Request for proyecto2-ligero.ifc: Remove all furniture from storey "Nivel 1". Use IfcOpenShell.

First a look at what the model holds.

```python
import ifcopenshell
import ifcopenshell.util.element

model = ifcopenshell.open("proyecto2-ligero.ifc")
print(model.schema)
storey = next(s for s in model.by_type("IfcBuildingStorey") if s.Name == "Nivel 1")
furniture = [e for e in ifcopenshell.util.element.get_decomposition(storey) if e.is_a("IfcFurnishingElement")]
seen = {}
for e in furniture:
    element_type = ifcopenshell.util.element.get_type(e)
    name = element_type.Name if element_type not in (None, e) else None
    seen[name] = seen.get(name, 0) + 1
for name, count in sorted(seen.items(), key=str):
    print(count, "x", name)
```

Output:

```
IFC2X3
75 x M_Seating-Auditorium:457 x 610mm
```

```python
import ifcopenshell
import ifcopenshell.api.root
import ifcopenshell.util.element

model = ifcopenshell.open("proyecto2-ligero.ifc")

storey = next(s for s in model.by_type("IfcBuildingStorey") if s.Name == "Nivel 1")
furniture = [e for e in ifcopenshell.util.element.get_decomposition(storey) if e.is_a("IfcFurnishingElement")]

for e in furniture:
    ifcopenshell.api.root.remove_product(model, product=e)
print(len(furniture), "removed")

model.write("proyecto2-ligero_rev.ifc")
```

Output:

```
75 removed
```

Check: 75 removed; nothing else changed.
